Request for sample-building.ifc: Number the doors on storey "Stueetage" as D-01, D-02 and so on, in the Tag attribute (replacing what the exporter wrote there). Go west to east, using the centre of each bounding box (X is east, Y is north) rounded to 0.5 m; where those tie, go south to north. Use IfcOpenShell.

First a look at what the model holds.

```python
import ifcopenshell
import ifcopenshell.util.element
import ifcopenshell.util.placement

model = ifcopenshell.open("sample-building.ifc")
print(model.schema)
storey = next(s for s in model.by_type("IfcBuildingStorey") if s.Name == "Stueetage")
doors = [e for e in ifcopenshell.util.element.get_decomposition(storey) if e.is_a("IfcDoor")]
for e in sorted(doors, key=lambda e: e.id()):
    origin = ifcopenshell.util.placement.get_local_placement(e.ObjectPlacement)[:3, 3]
    print(e.id(), e.Tag, e.Name, origin.round(2) + 0.0, sep=" | ")
```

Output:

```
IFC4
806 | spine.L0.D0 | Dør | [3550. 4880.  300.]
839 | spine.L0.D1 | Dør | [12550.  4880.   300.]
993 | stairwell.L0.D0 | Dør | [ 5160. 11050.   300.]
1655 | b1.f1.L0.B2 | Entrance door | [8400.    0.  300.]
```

```python
import ifcopenshell
import ifcopenshell.geom
import ifcopenshell.util.element
import ifcopenshell.util.shape

model = ifcopenshell.open("sample-building.ifc")
settings = ifcopenshell.geom.settings()
settings.set("use-world-coords", True)


def centre(element):
    shape = ifcopenshell.geom.create_shape(settings, element)
    return ifcopenshell.util.shape.get_bbox_centroid(shape.geometry)


storey = next(s for s in model.by_type("IfcBuildingStorey") if s.Name == "Stueetage")
doors = [e for e in ifcopenshell.util.element.get_decomposition(storey) if e.is_a("IfcDoor")]

# Insertion points can sit at a corner or the storey origin, so sort by the geometry (in metres).
centres = {e: centre(e) for e in doors}
doors.sort(key=lambda e: (round(centres[e][0] / 0.5), centres[e][1]))

for i, e in enumerate(doors, start=1):
    number = f"D-{i:02d}"
    e.Tag = number
    print(e.id(), number)

model.write("sample-building_updated.ifc")
```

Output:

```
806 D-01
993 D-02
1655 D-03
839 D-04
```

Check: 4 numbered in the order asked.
